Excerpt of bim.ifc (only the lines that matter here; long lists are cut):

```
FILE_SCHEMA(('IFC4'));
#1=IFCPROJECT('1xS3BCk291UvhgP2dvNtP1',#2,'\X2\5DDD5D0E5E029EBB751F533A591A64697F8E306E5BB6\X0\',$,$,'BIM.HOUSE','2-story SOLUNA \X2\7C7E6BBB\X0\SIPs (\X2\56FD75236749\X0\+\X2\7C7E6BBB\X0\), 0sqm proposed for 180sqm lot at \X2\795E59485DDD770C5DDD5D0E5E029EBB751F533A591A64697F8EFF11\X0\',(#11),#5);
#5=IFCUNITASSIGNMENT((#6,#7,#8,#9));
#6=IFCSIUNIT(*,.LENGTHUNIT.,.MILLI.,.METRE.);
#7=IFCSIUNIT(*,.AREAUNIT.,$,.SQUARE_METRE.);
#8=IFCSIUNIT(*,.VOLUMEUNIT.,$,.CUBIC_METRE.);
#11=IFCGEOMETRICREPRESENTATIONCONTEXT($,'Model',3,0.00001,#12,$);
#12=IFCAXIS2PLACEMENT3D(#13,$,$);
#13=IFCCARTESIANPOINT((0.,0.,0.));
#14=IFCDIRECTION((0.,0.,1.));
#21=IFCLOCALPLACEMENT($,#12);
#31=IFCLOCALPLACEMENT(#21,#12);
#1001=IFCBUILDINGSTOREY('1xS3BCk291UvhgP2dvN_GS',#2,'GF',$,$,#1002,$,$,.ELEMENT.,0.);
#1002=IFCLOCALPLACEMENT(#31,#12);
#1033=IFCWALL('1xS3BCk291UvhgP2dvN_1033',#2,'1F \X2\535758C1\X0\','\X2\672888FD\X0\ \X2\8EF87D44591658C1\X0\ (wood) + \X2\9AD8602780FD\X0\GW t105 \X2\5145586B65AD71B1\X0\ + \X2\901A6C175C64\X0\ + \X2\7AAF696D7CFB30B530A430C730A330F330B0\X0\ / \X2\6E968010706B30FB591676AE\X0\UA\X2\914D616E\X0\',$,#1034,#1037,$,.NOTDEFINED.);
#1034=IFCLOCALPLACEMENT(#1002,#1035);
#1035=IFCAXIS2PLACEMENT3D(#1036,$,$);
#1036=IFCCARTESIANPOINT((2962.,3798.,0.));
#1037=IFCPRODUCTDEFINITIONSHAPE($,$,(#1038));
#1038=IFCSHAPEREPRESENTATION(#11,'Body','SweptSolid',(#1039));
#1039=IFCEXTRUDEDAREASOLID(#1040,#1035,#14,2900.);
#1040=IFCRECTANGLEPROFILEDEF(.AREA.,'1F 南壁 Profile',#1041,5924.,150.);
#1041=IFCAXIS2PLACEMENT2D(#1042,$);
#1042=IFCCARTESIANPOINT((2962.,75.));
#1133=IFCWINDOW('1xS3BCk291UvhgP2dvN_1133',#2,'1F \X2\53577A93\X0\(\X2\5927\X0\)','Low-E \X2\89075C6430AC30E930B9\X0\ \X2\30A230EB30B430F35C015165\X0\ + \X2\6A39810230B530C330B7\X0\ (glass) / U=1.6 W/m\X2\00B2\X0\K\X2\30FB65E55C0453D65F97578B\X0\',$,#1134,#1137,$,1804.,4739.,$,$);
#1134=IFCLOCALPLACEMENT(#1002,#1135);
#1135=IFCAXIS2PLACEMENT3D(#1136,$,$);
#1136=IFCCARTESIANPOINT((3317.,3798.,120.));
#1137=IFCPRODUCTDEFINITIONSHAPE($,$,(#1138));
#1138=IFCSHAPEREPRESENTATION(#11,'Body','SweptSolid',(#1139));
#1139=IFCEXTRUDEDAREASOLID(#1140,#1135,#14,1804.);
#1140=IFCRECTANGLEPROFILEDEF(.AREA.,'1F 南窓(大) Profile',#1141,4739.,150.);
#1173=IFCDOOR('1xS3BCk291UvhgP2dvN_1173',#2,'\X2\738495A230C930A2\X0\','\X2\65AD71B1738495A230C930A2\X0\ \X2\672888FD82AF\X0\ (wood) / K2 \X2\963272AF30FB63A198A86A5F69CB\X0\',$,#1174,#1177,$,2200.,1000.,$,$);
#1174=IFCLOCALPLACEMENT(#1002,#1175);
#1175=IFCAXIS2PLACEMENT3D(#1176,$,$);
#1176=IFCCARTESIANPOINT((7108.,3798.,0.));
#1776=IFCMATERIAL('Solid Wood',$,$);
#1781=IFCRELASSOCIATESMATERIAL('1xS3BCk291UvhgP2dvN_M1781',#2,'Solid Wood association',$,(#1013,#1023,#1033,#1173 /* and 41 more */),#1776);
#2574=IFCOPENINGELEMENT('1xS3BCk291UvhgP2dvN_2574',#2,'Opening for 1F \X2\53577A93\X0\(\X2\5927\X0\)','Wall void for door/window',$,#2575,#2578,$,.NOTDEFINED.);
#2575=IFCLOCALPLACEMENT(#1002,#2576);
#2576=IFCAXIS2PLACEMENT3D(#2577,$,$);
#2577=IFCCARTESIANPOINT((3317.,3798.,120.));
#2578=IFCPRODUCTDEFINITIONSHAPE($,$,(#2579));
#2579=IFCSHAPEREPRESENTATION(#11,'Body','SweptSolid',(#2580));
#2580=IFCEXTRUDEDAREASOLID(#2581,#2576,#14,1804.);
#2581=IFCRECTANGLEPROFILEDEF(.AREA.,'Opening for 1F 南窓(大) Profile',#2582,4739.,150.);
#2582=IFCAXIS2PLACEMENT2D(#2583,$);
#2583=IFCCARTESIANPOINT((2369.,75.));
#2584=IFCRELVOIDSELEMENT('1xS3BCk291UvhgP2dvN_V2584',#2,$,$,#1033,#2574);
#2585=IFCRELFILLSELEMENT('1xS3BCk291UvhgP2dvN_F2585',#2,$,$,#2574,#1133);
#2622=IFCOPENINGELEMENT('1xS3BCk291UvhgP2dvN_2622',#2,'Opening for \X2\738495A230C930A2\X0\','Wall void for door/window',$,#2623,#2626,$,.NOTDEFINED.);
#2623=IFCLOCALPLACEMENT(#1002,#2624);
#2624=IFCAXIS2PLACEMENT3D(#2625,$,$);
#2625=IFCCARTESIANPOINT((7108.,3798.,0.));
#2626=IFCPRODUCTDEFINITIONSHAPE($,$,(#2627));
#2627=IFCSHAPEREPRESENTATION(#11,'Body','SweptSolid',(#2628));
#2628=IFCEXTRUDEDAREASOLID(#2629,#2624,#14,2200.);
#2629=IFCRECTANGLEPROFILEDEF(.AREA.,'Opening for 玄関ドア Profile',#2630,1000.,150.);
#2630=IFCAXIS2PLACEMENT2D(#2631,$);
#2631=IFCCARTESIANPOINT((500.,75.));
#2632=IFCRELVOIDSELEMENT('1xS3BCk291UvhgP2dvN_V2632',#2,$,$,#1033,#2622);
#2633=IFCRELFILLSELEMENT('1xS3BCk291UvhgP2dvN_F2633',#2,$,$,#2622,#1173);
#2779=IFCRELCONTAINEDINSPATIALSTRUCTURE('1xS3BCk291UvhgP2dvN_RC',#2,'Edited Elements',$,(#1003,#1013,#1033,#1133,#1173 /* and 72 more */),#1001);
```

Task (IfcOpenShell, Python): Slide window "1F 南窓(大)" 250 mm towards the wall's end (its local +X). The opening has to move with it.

```python
import ifcopenshell
import ifcopenshell.api.geometry
import ifcopenshell.util.placement

model = ifcopenshell.open("bim.ifc")

window = model.by_guid("1xS3BCk291UvhgP2dvN_1133")
opening = window.FillsVoids[0].RelatingOpeningElement
wall = opening.VoidsElements[0].RelatingBuildingElement

wall_matrix = ifcopenshell.util.placement.get_local_placement(wall.ObjectPlacement)
shift = wall_matrix[:3, 0] * 250.0
before = ifcopenshell.util.placement.get_local_placement(window.ObjectPlacement)[:3, 3].copy()

# The window is not placed relative to its opening, so move both.
for product in (opening, window):
    matrix = ifcopenshell.util.placement.get_local_placement(product.ObjectPlacement)
    matrix[:3, 3] += shift
    ifcopenshell.api.geometry.edit_object_placement(model, product=product, matrix=matrix, is_si=False)

after = ifcopenshell.util.placement.get_local_placement(window.ObjectPlacement)[:3, 3]
print("window moved by", (after - before).round(3) + 0.0)

model.write("bim_updated.ifc")
```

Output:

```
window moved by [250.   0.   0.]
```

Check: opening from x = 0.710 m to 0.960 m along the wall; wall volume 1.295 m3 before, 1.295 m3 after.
